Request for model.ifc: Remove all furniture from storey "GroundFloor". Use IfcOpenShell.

First a look at what the model holds.

```python
import ifcopenshell
import ifcopenshell.util.element

model = ifcopenshell.open("model.ifc")
print(model.schema)
storey = next(s for s in model.by_type("IfcBuildingStorey") if s.Name == "GroundFloor")
furniture = [e for e in ifcopenshell.util.element.get_decomposition(storey) if e.is_a("IfcFurnishingElement")]
seen = {}
for e in furniture:
    element_type = ifcopenshell.util.element.get_type(e)
    name = element_type.Name if element_type not in (None, e) else None
    seen[name] = seen.get(name, 0) + 1
for name, count in sorted(seen.items(), key=str):
    print(count, "x", name)
```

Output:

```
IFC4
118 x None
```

```python
import ifcopenshell
import ifcopenshell.api.root
import ifcopenshell.util.element

model = ifcopenshell.open("model.ifc")

storey = next(s for s in model.by_type("IfcBuildingStorey") if s.Name == "GroundFloor")
furniture = [e for e in ifcopenshell.util.element.get_decomposition(storey) if e.is_a("IfcFurnishingElement")]

for e in furniture:
    ifcopenshell.api.root.remove_product(model, product=e)
print(len(furniture), "removed")

model.write("model_v2.ifc")
```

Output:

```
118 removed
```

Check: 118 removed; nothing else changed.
